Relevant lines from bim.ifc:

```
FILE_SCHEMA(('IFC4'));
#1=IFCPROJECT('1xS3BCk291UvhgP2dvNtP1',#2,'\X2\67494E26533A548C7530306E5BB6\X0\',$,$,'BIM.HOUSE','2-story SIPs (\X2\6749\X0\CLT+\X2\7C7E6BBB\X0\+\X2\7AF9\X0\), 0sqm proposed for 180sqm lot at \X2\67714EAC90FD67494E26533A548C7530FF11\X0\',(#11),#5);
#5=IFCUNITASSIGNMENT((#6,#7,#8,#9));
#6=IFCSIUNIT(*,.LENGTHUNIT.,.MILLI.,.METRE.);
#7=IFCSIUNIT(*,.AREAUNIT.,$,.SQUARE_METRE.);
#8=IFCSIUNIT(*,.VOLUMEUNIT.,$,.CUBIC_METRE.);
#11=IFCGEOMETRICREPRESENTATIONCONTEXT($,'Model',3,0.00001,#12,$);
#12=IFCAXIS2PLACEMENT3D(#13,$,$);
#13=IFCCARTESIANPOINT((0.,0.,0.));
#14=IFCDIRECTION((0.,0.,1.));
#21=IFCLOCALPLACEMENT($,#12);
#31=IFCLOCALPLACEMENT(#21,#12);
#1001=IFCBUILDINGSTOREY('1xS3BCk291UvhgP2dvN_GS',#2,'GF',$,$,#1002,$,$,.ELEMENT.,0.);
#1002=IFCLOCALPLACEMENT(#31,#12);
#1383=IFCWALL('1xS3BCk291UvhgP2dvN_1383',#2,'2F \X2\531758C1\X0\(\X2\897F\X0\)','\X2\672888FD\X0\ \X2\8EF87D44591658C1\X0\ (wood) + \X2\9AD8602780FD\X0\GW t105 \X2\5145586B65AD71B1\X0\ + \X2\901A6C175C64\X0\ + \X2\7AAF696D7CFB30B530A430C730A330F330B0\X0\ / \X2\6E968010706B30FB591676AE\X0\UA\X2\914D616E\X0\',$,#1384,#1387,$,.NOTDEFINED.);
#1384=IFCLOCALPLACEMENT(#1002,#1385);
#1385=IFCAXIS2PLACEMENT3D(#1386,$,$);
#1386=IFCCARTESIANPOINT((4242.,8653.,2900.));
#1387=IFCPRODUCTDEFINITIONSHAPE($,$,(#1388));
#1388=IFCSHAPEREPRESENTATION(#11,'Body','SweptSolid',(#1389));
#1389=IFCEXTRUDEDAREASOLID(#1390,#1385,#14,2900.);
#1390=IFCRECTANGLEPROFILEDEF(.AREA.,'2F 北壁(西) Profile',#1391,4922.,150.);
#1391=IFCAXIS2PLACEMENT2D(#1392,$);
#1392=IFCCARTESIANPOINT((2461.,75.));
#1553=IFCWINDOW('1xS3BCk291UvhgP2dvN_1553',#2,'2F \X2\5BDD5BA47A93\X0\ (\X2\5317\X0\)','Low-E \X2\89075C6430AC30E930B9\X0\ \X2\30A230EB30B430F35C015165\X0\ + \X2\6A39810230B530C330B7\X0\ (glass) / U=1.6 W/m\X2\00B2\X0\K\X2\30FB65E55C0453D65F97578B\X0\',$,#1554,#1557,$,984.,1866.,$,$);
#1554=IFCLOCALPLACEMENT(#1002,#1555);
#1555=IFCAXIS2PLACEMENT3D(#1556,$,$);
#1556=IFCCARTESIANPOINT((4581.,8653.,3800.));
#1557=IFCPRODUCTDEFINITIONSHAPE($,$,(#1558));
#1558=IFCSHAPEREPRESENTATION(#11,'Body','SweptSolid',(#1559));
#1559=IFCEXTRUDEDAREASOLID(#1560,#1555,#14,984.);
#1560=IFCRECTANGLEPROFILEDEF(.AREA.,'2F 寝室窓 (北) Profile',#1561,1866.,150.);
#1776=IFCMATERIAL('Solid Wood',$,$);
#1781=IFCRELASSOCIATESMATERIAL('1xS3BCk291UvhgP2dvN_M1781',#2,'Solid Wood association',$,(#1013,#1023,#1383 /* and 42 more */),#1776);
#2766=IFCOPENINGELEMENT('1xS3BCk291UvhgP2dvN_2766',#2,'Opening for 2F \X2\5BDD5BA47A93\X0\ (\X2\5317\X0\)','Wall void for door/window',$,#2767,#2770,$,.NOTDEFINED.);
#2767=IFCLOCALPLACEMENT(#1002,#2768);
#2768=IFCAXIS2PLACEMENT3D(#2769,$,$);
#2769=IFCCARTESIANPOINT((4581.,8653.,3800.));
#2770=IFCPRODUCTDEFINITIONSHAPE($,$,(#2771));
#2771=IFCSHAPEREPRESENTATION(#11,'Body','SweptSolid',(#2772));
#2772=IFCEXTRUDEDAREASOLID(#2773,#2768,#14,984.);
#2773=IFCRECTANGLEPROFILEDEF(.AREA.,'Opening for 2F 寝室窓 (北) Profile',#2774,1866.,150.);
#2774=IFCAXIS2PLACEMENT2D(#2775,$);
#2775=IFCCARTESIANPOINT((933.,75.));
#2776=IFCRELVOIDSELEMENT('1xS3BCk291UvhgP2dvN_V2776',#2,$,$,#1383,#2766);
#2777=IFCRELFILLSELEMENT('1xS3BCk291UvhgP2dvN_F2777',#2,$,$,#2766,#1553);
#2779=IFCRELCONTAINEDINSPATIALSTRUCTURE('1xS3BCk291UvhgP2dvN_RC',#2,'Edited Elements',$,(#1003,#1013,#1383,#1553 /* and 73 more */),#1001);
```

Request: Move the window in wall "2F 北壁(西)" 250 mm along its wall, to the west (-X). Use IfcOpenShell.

```python
import ifcopenshell
import ifcopenshell.api.geometry
import ifcopenshell.util.placement

model = ifcopenshell.open("bim.ifc")

window = model.by_guid("1xS3BCk291UvhgP2dvN_1553")
opening = window.FillsVoids[0].RelatingOpeningElement
wall = opening.VoidsElements[0].RelatingBuildingElement

wall_matrix = ifcopenshell.util.placement.get_local_placement(wall.ObjectPlacement)
shift = wall_matrix[:3, 0] * -250.0
before = ifcopenshell.util.placement.get_local_placement(window.ObjectPlacement)[:3, 3].copy()

# The window is not placed relative to its opening, so move both.
for product in (opening, window):
    matrix = ifcopenshell.util.placement.get_local_placement(product.ObjectPlacement)
    matrix[:3, 3] += shift
    ifcopenshell.api.geometry.edit_object_placement(model, product=product, matrix=matrix, is_si=False)

after = ifcopenshell.util.placement.get_local_placement(window.ObjectPlacement)[:3, 3]
print("window moved by", (after - before).round(3) + 0.0)

model.write("bim_v2.ifc")
```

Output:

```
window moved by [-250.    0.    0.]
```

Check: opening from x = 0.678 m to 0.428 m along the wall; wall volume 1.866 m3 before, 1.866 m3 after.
